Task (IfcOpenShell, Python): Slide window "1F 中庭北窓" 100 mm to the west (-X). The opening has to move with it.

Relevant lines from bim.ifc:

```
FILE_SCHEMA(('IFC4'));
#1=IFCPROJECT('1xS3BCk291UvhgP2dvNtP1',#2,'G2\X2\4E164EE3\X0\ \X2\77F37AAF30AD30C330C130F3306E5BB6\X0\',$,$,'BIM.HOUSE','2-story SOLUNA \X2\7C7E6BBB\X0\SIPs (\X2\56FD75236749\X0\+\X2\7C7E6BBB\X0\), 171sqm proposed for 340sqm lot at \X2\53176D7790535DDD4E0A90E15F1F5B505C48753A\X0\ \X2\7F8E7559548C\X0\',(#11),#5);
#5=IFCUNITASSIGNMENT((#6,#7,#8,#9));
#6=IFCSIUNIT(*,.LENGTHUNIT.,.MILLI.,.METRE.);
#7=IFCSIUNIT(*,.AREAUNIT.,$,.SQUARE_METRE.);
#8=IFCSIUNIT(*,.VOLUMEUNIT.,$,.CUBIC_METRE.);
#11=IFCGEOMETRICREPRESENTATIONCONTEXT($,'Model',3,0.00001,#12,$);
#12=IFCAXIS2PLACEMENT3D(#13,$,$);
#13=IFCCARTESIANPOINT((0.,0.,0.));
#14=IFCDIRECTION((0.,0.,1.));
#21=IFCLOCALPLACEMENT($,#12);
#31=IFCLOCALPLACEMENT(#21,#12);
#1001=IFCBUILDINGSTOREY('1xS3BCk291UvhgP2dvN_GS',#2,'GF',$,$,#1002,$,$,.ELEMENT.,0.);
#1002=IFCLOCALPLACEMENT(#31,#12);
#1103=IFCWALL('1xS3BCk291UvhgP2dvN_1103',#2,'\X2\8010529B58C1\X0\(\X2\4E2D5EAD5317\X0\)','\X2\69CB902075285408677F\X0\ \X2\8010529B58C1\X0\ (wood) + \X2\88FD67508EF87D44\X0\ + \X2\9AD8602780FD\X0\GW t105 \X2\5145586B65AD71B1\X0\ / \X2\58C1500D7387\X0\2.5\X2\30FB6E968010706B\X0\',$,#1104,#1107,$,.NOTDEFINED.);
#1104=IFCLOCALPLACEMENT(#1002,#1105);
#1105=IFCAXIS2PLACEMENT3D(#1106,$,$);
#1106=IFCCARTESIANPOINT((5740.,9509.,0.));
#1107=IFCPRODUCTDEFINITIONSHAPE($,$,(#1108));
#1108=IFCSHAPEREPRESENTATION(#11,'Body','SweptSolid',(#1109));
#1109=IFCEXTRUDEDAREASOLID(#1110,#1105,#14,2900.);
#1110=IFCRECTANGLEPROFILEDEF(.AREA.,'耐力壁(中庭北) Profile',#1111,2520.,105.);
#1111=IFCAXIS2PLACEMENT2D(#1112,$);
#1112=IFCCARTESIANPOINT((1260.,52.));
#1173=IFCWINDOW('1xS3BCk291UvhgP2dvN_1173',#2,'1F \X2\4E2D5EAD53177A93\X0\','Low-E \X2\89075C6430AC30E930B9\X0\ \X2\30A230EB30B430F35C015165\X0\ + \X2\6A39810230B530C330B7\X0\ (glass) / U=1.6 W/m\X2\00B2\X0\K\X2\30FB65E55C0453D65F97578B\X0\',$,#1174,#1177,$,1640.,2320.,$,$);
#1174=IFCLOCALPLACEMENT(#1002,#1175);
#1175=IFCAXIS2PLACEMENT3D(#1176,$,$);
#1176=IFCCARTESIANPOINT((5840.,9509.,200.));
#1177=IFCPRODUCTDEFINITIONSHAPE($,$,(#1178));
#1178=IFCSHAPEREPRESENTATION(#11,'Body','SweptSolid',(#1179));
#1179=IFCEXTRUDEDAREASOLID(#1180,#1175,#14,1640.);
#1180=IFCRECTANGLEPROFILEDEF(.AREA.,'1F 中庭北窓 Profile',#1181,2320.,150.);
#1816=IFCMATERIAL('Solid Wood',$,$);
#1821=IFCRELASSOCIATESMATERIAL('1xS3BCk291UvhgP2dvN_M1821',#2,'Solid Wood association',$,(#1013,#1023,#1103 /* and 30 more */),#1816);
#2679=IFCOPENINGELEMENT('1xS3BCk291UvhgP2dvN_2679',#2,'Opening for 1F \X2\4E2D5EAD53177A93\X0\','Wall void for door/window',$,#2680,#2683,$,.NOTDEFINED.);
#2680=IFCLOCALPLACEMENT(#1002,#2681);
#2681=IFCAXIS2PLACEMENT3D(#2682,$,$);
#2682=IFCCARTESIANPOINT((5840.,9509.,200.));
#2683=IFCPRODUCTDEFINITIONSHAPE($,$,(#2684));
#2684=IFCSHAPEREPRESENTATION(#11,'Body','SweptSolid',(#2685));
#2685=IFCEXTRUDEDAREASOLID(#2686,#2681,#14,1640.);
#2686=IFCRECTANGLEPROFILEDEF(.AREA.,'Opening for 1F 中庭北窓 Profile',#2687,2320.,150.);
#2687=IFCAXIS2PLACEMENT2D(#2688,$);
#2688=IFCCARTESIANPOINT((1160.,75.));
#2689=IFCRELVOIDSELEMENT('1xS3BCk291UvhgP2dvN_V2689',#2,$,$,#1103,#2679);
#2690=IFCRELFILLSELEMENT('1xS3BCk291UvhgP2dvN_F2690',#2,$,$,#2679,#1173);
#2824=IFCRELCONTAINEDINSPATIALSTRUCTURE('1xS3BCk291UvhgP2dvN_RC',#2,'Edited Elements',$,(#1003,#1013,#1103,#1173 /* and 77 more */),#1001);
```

```python
import ifcopenshell
import ifcopenshell.api.geometry
import ifcopenshell.util.placement

model = ifcopenshell.open("bim.ifc")

window = model.by_id(1173)
opening = window.FillsVoids[0].RelatingOpeningElement
wall = opening.VoidsElements[0].RelatingBuildingElement

wall_matrix = ifcopenshell.util.placement.get_local_placement(wall.ObjectPlacement)
shift = wall_matrix[:3, 0] * -100.0
before = ifcopenshell.util.placement.get_local_placement(window.ObjectPlacement)[:3, 3].copy()

# The window is not placed relative to its opening, so move both.
for product in (opening, window):
    matrix = ifcopenshell.util.placement.get_local_placement(product.ObjectPlacement)
    matrix[:3, 3] += shift
    ifcopenshell.api.geometry.edit_object_placement(model, product=product, matrix=matrix, is_si=False)

after = ifcopenshell.util.placement.get_local_placement(window.ObjectPlacement)[:3, 3]
print("window moved by", (after - before).round(3) + 0.0)

model.write("bim_updated.ifc")
```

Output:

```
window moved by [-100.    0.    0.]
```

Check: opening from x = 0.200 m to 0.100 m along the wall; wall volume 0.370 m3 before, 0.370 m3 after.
